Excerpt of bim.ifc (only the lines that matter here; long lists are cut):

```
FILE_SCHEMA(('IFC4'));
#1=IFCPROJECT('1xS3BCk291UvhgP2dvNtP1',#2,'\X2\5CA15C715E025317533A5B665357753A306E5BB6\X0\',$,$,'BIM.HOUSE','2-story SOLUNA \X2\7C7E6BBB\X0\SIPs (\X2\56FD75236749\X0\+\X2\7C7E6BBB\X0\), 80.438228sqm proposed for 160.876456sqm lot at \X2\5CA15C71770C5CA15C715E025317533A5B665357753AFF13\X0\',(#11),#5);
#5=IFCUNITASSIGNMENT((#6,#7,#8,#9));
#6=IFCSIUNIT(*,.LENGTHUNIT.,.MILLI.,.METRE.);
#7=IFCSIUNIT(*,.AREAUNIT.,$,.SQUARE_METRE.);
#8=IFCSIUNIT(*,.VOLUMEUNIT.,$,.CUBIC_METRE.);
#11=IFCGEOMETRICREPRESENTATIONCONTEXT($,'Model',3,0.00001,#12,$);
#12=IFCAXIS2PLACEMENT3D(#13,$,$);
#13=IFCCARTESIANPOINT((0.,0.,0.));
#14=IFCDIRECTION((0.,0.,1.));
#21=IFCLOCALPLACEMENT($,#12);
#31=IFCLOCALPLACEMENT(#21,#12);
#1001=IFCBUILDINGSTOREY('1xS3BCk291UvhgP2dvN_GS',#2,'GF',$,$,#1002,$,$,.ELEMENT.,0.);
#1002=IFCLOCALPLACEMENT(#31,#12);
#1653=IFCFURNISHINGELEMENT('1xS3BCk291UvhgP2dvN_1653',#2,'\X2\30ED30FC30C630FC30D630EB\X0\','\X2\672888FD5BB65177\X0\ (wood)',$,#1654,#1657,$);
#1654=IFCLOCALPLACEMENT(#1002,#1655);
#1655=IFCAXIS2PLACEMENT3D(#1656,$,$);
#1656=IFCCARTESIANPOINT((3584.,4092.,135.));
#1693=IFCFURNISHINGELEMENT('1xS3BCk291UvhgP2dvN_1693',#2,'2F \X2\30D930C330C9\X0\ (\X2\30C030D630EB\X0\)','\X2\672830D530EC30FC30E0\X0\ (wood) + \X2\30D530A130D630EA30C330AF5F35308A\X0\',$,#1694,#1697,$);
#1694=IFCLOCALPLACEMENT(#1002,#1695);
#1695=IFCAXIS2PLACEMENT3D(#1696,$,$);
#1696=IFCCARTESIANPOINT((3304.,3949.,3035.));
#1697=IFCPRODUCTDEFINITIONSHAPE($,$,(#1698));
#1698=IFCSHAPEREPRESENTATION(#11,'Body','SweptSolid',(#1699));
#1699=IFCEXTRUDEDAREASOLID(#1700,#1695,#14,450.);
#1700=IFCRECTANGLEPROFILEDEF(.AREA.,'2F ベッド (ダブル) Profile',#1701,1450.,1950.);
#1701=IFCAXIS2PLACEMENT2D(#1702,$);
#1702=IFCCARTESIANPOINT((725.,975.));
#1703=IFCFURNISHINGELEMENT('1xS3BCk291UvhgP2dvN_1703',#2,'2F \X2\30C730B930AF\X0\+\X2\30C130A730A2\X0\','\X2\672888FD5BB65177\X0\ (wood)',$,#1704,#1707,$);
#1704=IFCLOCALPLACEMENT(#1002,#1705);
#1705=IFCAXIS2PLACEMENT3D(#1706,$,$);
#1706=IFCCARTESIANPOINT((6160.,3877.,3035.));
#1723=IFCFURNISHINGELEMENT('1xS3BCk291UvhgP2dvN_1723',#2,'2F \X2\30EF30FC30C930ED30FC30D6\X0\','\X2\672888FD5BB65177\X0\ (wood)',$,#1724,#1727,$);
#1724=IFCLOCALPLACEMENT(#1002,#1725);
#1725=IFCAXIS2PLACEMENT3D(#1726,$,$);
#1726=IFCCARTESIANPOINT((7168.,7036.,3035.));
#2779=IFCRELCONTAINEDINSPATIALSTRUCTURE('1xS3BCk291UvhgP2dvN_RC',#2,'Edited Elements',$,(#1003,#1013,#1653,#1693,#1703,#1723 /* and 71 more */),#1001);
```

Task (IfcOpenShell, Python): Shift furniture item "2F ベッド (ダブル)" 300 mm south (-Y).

```python
import ifcopenshell
import ifcopenshell.api.geometry
import ifcopenshell.util.placement
import ifcopenshell.util.unit

model = ifcopenshell.open("bim.ifc")
unit_scale = ifcopenshell.util.unit.calculate_unit_scale(model)

item = model.by_id(1693)
matrix = ifcopenshell.util.placement.get_local_placement(item.ObjectPlacement)
matrix[1, 3] -= 0.3 / unit_scale
ifcopenshell.api.geometry.edit_object_placement(model, product=item, matrix=matrix, is_si=False)

print(ifcopenshell.util.placement.get_local_placement(item.ObjectPlacement).round(3) + 0.0)

model.write("bim_v2.ifc")
```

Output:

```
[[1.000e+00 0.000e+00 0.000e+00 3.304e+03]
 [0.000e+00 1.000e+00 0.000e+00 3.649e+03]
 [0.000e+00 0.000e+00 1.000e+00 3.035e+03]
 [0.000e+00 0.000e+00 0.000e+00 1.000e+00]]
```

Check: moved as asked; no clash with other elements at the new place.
